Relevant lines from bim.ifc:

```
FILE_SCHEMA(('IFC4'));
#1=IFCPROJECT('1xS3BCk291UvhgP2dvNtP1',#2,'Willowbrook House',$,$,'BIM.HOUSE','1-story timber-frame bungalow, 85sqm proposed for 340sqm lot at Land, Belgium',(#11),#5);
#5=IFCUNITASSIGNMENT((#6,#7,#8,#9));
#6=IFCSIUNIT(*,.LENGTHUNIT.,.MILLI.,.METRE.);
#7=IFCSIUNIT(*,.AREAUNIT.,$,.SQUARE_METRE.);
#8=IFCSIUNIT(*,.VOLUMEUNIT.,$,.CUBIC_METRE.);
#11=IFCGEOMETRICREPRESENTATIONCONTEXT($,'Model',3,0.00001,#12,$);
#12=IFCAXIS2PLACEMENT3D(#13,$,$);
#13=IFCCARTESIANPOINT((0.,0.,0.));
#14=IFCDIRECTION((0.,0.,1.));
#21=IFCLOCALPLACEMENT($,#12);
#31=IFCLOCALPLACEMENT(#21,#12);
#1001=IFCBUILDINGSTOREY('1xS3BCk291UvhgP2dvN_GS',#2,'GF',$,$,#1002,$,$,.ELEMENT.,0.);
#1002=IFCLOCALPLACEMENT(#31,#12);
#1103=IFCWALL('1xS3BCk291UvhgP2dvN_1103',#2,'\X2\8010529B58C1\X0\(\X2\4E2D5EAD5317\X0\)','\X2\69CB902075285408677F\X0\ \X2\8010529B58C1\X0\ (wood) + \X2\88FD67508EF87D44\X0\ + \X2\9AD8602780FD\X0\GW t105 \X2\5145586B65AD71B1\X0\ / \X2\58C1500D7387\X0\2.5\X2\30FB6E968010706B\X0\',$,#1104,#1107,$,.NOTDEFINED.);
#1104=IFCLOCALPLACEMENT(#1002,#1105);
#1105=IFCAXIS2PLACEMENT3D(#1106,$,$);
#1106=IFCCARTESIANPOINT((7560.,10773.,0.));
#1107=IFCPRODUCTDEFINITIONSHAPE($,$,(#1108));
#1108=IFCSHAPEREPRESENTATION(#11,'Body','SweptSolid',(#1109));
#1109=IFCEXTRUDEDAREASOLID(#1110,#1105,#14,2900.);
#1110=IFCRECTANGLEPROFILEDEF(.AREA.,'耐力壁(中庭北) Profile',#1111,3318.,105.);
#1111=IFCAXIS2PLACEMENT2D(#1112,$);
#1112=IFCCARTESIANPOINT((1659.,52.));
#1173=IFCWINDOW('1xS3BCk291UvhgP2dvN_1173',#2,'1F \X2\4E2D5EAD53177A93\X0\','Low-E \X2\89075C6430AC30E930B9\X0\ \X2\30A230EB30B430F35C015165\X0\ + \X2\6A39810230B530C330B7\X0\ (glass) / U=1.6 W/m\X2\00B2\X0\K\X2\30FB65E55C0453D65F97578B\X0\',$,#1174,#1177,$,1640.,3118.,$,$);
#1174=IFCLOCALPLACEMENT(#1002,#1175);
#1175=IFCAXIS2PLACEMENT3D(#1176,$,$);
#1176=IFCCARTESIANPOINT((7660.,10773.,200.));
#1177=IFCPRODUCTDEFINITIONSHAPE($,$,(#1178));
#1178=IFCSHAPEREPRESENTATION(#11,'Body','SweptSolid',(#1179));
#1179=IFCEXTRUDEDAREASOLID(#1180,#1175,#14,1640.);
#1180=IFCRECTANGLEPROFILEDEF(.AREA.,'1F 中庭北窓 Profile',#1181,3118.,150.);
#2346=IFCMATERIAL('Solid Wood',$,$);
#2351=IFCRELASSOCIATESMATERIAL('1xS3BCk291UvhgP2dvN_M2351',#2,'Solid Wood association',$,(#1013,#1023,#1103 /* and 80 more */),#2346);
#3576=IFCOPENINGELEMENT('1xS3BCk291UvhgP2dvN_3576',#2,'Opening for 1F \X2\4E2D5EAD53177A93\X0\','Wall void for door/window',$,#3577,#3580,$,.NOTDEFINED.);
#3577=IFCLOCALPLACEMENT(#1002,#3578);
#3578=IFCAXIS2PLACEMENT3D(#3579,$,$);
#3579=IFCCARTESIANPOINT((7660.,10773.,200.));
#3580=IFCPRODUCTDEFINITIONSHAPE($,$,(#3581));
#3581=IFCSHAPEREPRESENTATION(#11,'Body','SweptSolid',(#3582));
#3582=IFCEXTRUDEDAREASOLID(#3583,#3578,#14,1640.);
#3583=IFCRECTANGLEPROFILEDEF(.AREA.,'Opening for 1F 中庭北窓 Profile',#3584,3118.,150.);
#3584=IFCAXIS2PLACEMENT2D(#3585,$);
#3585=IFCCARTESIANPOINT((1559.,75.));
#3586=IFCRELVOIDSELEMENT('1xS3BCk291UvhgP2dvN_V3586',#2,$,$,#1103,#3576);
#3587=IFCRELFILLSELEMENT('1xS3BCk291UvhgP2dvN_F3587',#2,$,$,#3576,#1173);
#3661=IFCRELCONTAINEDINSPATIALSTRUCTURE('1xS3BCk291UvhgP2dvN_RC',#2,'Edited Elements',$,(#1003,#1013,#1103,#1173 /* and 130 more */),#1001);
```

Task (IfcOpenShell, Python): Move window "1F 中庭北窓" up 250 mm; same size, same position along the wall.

```python
import numpy as np
import ifcopenshell
import ifcopenshell.api.geometry
import ifcopenshell.util.placement
import ifcopenshell.util.unit

model = ifcopenshell.open("bim.ifc")
unit_scale = ifcopenshell.util.unit.calculate_unit_scale(model)

window = model.by_guid("1xS3BCk291UvhgP2dvN_1173")
opening = window.FillsVoids[0].RelatingOpeningElement
dz = 0.25 / unit_scale

shift = np.array([0.0, 0.0, dz])
# The window is not placed relative to its opening, so move both.
for product in (opening, window):
    matrix = ifcopenshell.util.placement.get_local_placement(product.ObjectPlacement)
    matrix[:3, 3] += shift
    ifcopenshell.api.geometry.edit_object_placement(model, product=product, matrix=matrix, is_si=False)

print(f"moved by {dz * unit_scale:+.3f} m")

model.write("bim_rev.ifc")
```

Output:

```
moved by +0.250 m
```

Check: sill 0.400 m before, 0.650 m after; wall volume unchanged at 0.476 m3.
